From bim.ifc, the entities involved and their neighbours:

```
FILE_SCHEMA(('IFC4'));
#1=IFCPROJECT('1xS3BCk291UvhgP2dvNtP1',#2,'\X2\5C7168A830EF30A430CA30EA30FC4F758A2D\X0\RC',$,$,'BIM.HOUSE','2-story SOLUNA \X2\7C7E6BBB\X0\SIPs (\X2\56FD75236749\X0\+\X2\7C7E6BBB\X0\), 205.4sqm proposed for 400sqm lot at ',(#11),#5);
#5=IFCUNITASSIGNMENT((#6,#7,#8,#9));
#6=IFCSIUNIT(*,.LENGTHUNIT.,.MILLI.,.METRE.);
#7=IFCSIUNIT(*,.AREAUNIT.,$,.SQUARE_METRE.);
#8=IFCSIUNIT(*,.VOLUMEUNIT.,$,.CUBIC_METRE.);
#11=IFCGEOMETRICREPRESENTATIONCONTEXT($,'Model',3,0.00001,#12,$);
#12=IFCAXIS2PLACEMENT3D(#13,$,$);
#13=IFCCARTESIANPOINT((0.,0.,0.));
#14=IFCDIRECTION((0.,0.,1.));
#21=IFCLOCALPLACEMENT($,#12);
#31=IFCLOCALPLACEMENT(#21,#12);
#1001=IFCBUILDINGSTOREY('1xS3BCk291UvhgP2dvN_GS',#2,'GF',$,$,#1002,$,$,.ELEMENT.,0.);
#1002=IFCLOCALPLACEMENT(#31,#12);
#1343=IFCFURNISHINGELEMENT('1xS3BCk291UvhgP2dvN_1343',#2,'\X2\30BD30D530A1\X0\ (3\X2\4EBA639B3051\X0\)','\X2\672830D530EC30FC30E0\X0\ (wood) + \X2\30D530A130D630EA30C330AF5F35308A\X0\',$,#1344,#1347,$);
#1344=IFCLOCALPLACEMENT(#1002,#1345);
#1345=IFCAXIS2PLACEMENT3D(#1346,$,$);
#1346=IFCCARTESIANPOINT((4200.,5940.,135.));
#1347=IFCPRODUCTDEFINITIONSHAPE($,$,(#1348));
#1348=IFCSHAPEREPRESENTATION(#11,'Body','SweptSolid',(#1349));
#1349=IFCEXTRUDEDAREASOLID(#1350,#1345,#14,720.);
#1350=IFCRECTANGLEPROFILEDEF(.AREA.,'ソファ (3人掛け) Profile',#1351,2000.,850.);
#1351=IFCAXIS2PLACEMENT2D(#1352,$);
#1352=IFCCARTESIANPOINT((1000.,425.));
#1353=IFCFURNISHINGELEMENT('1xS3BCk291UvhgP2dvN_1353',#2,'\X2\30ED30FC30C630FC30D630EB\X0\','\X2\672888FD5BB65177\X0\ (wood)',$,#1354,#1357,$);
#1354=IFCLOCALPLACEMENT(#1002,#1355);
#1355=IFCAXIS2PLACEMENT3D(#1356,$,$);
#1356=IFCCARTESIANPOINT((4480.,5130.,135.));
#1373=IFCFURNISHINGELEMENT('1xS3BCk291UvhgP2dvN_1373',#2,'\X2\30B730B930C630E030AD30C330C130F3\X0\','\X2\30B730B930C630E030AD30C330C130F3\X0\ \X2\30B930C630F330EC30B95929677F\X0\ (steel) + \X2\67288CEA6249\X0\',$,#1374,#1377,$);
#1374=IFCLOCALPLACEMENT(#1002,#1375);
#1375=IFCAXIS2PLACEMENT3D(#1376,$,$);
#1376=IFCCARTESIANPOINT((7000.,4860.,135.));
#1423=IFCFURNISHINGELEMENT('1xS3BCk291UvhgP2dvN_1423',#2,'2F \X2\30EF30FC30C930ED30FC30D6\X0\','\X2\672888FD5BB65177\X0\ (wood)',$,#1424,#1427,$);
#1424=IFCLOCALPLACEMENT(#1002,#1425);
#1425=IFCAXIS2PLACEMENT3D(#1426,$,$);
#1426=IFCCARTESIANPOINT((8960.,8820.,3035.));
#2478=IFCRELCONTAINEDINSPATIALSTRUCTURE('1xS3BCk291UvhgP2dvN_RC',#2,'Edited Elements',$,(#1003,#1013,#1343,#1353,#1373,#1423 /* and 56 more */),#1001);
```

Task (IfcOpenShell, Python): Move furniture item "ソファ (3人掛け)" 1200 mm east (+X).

```python
import ifcopenshell
import ifcopenshell.api.geometry
import ifcopenshell.util.placement

model = ifcopenshell.open("bim.ifc")

item = model.by_guid("1xS3BCk291UvhgP2dvN_1343")
matrix = ifcopenshell.util.placement.get_local_placement(item.ObjectPlacement)
matrix[0, 3] += 1200.0
ifcopenshell.api.geometry.edit_object_placement(model, product=item, matrix=matrix, is_si=False)

print(ifcopenshell.util.placement.get_local_placement(item.ObjectPlacement).round(3) + 0.0)

model.write("bim_rev.ifc")
```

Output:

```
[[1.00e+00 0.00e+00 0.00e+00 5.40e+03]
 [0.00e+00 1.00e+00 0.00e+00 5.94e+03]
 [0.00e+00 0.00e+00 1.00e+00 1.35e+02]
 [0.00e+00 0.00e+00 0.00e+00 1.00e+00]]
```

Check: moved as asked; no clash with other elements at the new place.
